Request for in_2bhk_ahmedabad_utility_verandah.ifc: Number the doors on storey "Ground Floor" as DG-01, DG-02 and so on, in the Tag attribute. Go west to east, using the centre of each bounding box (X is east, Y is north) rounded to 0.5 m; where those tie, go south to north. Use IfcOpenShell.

First a look at what the model holds.

```python
import ifcopenshell
import ifcopenshell.util.element
import ifcopenshell.util.placement

model = ifcopenshell.open("in_2bhk_ahmedabad_utility_verandah.ifc")
print(model.schema)
storey = next(s for s in model.by_type("IfcBuildingStorey") if s.Name == "Ground Floor")
doors = [e for e in ifcopenshell.util.element.get_decomposition(storey) if e.is_a("IfcDoor")]
for e in sorted(doors, key=lambda e: e.id()):
    origin = ifcopenshell.util.placement.get_local_placement(e.ObjectPlacement)[:3, 3]
    print(e.id(), e.Tag, e.Name, origin.round(2) + 0.0, sep=" | ")
```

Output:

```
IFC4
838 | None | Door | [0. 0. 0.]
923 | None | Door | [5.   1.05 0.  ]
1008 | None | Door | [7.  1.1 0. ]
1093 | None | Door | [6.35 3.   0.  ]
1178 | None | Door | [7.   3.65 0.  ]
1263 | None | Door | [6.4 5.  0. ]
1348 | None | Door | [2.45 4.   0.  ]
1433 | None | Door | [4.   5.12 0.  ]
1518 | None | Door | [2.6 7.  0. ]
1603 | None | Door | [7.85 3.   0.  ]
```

```python
import ifcopenshell
import ifcopenshell.geom
import ifcopenshell.util.element
import ifcopenshell.util.shape

model = ifcopenshell.open("in_2bhk_ahmedabad_utility_verandah.ifc")
settings = ifcopenshell.geom.settings()
settings.set("use-world-coords", True)


def centre(element):
    shape = ifcopenshell.geom.create_shape(settings, element)
    return ifcopenshell.util.shape.get_bbox_centroid(shape.geometry)


storey = next(s for s in model.by_type("IfcBuildingStorey") if s.Name == "Ground Floor")
doors = [e for e in ifcopenshell.util.element.get_decomposition(storey) if e.is_a("IfcDoor")]

# Insertion points can sit at a corner or the storey origin, so sort by the geometry (in metres).
centres = {e: centre(e) for e in doors}
doors.sort(key=lambda e: (round(centres[e][0] / 0.5), centres[e][1]))

for i, e in enumerate(doors, start=1):
    number = f"DG-{i:02d}"
    e.Tag = number
    print(e.id(), number)

model.write("in_2bhk_ahmedabad_utility_verandah_edited.ifc")
```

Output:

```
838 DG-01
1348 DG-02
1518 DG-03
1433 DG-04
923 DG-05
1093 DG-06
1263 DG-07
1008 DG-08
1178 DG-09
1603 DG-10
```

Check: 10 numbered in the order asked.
